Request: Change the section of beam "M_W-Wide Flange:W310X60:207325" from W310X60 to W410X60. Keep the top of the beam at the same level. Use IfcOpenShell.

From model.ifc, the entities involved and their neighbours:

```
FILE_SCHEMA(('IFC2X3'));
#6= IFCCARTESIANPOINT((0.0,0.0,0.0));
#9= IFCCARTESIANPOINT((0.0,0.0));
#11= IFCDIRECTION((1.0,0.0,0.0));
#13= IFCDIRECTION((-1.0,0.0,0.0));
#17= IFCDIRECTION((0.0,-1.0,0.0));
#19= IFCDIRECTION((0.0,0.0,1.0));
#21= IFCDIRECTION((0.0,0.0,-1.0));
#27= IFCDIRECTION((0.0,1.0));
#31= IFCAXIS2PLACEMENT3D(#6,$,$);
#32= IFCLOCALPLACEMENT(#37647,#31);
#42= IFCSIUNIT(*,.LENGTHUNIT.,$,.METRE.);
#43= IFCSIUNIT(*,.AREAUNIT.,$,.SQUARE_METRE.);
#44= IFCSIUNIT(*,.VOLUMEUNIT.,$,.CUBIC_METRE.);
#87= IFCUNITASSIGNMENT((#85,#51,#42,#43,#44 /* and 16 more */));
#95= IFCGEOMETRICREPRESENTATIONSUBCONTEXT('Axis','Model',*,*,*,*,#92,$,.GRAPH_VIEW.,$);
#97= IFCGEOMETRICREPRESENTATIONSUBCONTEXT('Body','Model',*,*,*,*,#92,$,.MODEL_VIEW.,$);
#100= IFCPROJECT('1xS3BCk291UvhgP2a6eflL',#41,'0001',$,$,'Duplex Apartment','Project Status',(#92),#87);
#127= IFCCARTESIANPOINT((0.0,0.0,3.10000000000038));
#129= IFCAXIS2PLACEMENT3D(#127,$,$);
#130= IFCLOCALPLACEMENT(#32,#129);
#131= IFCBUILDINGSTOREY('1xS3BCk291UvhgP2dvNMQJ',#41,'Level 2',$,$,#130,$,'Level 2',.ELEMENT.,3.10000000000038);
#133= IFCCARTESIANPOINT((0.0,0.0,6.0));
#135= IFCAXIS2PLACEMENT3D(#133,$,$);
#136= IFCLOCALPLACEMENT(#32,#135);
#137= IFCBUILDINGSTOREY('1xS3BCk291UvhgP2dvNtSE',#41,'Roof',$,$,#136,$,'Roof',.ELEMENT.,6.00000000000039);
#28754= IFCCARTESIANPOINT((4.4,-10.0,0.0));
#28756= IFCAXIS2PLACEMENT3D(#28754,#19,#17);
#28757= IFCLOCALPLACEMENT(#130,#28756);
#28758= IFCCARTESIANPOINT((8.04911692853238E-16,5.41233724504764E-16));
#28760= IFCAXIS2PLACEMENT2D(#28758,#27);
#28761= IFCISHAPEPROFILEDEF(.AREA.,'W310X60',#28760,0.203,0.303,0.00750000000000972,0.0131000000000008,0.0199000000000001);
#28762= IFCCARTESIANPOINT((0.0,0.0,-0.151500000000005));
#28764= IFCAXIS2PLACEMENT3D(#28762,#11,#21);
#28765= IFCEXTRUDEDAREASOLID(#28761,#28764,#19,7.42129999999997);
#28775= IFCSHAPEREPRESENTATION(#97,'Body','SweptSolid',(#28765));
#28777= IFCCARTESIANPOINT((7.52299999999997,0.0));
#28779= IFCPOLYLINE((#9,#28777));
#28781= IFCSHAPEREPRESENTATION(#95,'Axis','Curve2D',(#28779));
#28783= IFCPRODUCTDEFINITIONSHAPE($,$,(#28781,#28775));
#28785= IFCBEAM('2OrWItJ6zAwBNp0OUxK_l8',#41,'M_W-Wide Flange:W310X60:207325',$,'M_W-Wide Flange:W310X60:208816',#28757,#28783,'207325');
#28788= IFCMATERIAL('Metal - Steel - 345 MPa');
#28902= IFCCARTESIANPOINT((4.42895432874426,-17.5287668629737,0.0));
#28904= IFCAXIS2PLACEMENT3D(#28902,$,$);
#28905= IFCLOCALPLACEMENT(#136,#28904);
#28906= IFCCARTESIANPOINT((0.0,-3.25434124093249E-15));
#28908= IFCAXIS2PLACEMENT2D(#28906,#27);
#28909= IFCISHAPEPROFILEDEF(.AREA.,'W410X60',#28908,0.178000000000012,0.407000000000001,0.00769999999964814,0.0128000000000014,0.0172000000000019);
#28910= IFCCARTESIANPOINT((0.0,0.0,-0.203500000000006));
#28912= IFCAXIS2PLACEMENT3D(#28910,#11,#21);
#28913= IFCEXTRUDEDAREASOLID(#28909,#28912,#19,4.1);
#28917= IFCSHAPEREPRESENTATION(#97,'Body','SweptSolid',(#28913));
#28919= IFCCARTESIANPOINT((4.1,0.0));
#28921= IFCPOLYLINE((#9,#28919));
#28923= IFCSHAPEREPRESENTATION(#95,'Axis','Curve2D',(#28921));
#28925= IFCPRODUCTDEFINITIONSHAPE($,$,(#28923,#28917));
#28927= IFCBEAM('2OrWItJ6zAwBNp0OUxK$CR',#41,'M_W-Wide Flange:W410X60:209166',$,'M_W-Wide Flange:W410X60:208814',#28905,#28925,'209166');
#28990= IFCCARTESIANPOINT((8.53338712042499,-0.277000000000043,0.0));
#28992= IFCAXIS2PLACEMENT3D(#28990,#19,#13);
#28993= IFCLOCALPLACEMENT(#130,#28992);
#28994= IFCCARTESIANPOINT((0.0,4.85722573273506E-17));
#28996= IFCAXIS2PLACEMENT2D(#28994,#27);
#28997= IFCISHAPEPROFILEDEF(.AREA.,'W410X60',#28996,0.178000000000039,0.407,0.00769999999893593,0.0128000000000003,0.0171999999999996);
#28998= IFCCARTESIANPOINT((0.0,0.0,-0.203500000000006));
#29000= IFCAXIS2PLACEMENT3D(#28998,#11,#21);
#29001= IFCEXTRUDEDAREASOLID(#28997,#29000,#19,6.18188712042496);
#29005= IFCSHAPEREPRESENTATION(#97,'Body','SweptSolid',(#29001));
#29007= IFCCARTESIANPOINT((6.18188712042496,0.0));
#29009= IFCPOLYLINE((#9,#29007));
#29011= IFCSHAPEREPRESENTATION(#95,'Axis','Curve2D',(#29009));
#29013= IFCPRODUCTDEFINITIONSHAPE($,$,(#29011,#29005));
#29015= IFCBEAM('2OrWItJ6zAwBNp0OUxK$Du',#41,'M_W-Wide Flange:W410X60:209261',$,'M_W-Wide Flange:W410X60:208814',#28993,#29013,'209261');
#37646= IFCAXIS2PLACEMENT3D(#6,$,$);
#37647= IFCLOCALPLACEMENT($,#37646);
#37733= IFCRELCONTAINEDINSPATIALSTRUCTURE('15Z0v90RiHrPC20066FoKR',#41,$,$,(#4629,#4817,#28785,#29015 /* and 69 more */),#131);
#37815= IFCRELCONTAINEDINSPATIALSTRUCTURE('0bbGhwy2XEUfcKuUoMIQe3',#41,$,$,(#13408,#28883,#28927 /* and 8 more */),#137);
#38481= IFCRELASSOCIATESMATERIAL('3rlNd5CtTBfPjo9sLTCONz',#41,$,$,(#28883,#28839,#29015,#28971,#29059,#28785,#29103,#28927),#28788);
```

```python
import ifcopenshell
import ifcopenshell.util.element
import ifcopenshell.util.representation

model = ifcopenshell.open("model.ifc")

member = model.by_guid("2OrWItJ6zAwBNp0OUxK_l8")
source = next(p for p in model.by_type("IfcIShapeProfileDef") if p.ProfileName == "W410X60")

body = ifcopenshell.util.representation.get_representation(member, "Model", "Body")
solid = body.Items[0]
old_profile = solid.SweptArea

# Copy the section's sizes but keep this member's own profile position.
profile = ifcopenshell.util.element.copy(model, source)
# Profiles are centred, so shift by half the change in depth to hold the top.
shift = (old_profile.OverallDepth - profile.OverallDepth) / 2
x, y = old_profile.Position.Location.Coordinates
up = (-1.0, 0.0)  # upwards, in the solid's own plane
location = model.createIfcCartesianPoint((x + up[0] * shift, y + up[1] * shift))
profile.Position = model.createIfcAxis2Placement2D(location, old_profile.Position.RefDirection)
solid.SweptArea = profile
if not model.get_total_inverses(old_profile):
    ifcopenshell.util.element.remove_deep2(model, old_profile)
member.Name = member.Name.replace("W310X60", "W410X60")
member.ObjectType = member.ObjectType.replace("W310X60", "W410X60")

print(solid.SweptArea)

model.write("model_edited.ifc")
```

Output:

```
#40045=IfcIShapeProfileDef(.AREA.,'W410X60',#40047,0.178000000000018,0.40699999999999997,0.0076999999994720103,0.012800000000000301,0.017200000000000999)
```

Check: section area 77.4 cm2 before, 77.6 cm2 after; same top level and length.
